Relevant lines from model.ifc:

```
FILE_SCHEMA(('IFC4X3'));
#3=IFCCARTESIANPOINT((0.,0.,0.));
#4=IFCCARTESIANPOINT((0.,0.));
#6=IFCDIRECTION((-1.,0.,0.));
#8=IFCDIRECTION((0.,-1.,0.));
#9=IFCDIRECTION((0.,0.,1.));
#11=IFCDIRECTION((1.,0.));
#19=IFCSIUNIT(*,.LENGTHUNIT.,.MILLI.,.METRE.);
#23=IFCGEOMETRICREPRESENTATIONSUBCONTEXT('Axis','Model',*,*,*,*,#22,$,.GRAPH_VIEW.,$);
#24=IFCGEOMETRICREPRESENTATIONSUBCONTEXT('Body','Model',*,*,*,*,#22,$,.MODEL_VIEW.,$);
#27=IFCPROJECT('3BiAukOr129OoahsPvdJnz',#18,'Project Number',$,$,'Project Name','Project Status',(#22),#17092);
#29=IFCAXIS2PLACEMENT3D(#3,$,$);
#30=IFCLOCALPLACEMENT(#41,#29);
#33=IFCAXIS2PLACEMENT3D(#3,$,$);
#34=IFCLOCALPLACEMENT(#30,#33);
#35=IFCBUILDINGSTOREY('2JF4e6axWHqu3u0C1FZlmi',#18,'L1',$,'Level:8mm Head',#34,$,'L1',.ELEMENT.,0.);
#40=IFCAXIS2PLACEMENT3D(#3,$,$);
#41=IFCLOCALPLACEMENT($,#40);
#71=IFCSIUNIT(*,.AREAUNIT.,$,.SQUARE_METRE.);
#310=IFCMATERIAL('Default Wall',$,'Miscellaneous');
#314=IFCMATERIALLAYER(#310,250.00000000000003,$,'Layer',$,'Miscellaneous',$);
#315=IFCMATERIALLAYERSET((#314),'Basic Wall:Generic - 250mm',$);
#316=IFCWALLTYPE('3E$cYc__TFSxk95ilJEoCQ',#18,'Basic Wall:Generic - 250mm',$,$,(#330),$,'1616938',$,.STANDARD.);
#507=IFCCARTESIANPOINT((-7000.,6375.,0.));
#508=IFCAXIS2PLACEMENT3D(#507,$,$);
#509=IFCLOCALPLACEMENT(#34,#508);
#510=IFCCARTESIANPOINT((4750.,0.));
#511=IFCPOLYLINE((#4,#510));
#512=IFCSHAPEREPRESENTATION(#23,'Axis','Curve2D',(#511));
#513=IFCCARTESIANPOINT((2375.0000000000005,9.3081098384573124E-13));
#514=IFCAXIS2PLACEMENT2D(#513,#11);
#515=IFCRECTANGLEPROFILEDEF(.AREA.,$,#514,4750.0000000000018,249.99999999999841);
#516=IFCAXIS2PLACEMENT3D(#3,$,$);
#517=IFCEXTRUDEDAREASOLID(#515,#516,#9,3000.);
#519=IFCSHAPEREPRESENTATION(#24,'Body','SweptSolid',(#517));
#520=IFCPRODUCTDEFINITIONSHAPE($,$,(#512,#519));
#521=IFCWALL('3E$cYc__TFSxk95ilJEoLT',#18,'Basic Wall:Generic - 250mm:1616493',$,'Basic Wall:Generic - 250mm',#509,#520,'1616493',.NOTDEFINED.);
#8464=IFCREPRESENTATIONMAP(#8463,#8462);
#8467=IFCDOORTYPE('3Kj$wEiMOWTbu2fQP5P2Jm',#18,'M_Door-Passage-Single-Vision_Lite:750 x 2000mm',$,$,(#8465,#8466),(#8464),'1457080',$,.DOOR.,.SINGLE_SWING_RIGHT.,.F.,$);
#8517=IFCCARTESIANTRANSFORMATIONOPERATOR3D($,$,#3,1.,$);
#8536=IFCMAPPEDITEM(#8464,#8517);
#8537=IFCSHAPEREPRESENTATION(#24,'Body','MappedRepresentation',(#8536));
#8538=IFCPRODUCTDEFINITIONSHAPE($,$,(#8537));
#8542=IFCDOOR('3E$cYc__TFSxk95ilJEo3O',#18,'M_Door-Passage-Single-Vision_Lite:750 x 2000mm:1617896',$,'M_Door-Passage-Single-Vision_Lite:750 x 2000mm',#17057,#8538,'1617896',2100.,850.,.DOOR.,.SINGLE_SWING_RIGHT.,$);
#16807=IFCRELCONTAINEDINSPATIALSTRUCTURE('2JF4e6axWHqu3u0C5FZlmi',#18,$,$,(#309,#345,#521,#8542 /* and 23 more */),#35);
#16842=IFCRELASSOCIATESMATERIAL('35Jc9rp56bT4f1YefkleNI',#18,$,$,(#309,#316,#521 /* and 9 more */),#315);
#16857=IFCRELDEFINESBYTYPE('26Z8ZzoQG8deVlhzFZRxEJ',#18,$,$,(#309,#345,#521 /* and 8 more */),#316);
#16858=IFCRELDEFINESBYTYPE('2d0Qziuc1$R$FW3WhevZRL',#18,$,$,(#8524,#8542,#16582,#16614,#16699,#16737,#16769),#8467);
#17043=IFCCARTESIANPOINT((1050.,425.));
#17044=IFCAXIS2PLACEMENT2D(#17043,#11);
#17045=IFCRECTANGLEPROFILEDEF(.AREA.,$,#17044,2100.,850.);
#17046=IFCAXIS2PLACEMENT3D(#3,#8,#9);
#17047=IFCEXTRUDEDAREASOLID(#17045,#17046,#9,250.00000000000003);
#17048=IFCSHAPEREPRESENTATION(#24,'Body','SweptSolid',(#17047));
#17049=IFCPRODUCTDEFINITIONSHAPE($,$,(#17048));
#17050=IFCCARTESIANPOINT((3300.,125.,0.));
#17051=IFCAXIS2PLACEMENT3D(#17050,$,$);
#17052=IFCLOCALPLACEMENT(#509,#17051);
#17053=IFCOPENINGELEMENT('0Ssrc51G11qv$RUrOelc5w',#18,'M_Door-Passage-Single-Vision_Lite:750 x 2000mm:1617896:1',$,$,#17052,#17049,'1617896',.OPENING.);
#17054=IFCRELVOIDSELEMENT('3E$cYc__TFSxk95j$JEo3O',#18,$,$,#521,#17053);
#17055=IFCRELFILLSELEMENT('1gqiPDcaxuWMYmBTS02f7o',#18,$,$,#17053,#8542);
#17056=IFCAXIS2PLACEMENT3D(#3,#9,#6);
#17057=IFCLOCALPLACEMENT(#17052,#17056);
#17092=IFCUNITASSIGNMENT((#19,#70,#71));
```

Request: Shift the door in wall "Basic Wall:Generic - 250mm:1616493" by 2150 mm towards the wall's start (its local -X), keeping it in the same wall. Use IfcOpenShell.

```python
import ifcopenshell
import ifcopenshell.api.geometry
import ifcopenshell.util.placement

model = ifcopenshell.open("model.ifc")

door = model.by_guid("3E$cYc__TFSxk95ilJEo3O")
opening = door.FillsVoids[0].RelatingOpeningElement
wall = opening.VoidsElements[0].RelatingBuildingElement

wall_matrix = ifcopenshell.util.placement.get_local_placement(wall.ObjectPlacement)
shift = wall_matrix[:3, 0] * -2150.0
before = ifcopenshell.util.placement.get_local_placement(door.ObjectPlacement)[:3, 3].copy()

# The door is placed relative to its opening, so it follows when the opening moves.
matrix = ifcopenshell.util.placement.get_local_placement(opening.ObjectPlacement)
matrix[:3, 3] += shift
ifcopenshell.api.geometry.edit_object_placement(
    model, product=opening, matrix=matrix, is_si=False, should_transform_children=True
)

after = ifcopenshell.util.placement.get_local_placement(door.ObjectPlacement)[:3, 3]
print("door moved by", (after - before).round(3) + 0.0)

model.write("model_edited.ifc")
```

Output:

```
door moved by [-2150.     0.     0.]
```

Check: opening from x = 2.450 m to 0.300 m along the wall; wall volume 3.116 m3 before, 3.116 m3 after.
